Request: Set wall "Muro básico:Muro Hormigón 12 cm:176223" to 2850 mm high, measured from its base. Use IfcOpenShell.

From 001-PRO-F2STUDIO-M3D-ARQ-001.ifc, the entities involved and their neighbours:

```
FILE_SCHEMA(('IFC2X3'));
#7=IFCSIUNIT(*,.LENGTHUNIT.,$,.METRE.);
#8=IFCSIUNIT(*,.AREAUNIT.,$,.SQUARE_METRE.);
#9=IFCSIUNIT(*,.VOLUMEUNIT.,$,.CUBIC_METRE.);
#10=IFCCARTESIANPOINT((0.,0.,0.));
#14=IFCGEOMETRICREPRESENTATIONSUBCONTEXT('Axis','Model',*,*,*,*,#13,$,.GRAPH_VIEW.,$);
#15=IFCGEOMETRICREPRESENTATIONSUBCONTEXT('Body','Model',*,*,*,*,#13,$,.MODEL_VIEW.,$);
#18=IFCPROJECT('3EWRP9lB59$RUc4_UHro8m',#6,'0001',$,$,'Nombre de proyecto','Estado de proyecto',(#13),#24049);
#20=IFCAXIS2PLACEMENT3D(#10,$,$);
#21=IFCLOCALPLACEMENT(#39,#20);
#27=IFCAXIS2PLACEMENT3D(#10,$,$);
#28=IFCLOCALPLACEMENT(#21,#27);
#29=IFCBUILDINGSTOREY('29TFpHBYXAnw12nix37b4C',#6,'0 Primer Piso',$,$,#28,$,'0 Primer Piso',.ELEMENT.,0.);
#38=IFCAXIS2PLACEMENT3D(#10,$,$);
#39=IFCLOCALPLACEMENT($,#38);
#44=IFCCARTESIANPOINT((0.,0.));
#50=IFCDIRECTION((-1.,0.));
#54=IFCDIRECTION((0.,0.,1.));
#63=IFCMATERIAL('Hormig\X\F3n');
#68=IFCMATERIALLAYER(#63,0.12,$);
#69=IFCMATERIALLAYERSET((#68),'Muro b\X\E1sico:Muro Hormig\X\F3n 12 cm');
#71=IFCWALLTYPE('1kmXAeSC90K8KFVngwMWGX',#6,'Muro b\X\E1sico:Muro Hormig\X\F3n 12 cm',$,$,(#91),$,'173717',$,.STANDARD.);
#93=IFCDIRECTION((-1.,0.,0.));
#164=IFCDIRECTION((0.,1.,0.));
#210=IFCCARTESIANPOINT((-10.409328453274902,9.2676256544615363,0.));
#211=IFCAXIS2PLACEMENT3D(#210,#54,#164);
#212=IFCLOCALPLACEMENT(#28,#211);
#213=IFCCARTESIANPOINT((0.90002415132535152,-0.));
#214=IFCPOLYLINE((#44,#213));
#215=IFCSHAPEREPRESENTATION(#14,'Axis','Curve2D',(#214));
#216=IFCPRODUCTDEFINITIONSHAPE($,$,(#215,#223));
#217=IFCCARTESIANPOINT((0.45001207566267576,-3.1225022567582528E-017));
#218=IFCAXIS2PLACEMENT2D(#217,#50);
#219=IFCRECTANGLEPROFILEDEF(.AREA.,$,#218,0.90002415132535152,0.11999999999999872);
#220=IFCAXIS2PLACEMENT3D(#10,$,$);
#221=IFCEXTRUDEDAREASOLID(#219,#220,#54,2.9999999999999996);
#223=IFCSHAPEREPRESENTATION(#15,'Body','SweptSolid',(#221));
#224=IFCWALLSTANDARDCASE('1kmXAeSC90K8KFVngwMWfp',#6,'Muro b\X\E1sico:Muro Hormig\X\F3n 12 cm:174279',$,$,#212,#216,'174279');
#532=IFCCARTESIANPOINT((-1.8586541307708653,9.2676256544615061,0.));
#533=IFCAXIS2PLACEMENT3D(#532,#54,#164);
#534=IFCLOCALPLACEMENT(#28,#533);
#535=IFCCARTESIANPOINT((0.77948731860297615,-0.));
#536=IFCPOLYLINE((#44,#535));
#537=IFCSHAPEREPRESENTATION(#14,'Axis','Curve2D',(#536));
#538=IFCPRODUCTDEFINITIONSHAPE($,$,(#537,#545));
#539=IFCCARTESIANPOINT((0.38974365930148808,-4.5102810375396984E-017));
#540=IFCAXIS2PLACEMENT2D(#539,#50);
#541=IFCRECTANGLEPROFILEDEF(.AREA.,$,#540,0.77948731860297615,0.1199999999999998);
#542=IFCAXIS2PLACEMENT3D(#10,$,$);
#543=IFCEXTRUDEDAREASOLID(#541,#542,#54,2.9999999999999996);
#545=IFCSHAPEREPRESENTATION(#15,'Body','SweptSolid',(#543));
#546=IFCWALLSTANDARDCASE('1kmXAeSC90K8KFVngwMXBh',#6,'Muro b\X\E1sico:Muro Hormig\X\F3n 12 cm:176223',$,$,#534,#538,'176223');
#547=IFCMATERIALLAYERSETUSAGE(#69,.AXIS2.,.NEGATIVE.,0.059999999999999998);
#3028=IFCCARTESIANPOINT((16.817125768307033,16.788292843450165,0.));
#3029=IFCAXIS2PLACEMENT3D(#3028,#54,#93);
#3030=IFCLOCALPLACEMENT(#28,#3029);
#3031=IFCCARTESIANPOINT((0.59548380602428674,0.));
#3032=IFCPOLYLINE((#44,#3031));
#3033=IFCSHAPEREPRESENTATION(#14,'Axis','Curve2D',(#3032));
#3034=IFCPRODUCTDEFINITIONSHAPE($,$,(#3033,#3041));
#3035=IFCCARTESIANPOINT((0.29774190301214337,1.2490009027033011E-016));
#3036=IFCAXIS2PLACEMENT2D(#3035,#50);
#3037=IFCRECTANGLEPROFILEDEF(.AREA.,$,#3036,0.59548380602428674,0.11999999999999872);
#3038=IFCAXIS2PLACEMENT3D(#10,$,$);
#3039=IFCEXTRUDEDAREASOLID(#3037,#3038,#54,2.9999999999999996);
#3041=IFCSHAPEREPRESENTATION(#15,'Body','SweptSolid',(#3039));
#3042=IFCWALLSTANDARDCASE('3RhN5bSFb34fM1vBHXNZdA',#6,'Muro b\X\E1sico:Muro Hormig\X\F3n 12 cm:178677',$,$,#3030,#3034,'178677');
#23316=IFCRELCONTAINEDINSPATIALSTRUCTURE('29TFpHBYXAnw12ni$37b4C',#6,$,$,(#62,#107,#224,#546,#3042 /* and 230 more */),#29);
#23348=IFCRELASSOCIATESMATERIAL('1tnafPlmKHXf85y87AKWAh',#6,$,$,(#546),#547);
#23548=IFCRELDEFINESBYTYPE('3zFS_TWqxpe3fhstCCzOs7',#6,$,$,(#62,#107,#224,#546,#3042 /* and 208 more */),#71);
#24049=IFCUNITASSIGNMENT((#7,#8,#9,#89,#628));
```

```python
import ifcopenshell
import ifcopenshell.geom
import ifcopenshell.util.representation
import ifcopenshell.util.shape
import ifcopenshell.util.unit

model = ifcopenshell.open("001-PRO-F2STUDIO-M3D-ARQ-001.ifc")
unit_scale = ifcopenshell.util.unit.calculate_unit_scale(model)
settings = ifcopenshell.geom.settings()


def volume(element):
    """Net volume in cubic metres, openings subtracted."""
    shape = ifcopenshell.geom.create_shape(settings, element)
    return ifcopenshell.util.shape.get_volume(shape.geometry)


wall = model.by_guid("1kmXAeSC90K8KFVngwMXBh")
before = volume(wall)

body = ifcopenshell.util.representation.get_representation(wall, "Model", "Body")
solid = body.Items[0]
old_height = solid.Depth
solid.Depth = 2.85 / unit_scale
after = volume(wall)

print(f"height {old_height:g} -> {solid.Depth:g}, volume {before:.3f} -> {after:.3f} m3")

model.write("001-PRO-F2STUDIO-M3D-ARQ-001_edited.ifc")
```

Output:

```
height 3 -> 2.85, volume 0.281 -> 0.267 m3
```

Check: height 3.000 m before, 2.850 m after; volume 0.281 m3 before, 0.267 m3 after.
